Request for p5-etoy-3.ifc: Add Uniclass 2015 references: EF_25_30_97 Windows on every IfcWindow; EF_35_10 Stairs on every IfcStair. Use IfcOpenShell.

First a look at what the model holds.

```python
import ifcopenshell

model = ifcopenshell.open("p5-etoy-3.ifc")
print(model.schema)
print("classifications:", [c.Name for c in model.by_type("IfcClassification")])
for ifc_class in ("IfcDoor", "IfcRoof", "IfcStair", "IfcWall", "IfcWindow"):
    print(ifc_class, len(model.by_type(ifc_class)))
```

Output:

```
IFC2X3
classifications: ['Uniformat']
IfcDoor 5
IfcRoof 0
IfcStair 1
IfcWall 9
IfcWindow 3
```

```python
import ifcopenshell
import ifcopenshell.api.classification

model = ifcopenshell.open("p5-etoy-3.ifc")

# IFC2X3 requires Source and Edition and has no link from the project to the system.
system = model.create_entity("IfcClassification", Source="NBS", Edition="2015", Name="Uniclass 2015")

codes = {
    "IfcWindow": ("EF_25_30_97", "Windows"),
    "IfcStair": ("EF_35_10", "Stairs"),
}
for ifc_class, (code, name) in codes.items():
    products = model.by_type(ifc_class)
    ifcopenshell.api.classification.add_reference(
        model, products=products, classification=system, identification=code, name=name
    )
    print(code, len(products))

model.write("p5-etoy-3_edited.ifc")
```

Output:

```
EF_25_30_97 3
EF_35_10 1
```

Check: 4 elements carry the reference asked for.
